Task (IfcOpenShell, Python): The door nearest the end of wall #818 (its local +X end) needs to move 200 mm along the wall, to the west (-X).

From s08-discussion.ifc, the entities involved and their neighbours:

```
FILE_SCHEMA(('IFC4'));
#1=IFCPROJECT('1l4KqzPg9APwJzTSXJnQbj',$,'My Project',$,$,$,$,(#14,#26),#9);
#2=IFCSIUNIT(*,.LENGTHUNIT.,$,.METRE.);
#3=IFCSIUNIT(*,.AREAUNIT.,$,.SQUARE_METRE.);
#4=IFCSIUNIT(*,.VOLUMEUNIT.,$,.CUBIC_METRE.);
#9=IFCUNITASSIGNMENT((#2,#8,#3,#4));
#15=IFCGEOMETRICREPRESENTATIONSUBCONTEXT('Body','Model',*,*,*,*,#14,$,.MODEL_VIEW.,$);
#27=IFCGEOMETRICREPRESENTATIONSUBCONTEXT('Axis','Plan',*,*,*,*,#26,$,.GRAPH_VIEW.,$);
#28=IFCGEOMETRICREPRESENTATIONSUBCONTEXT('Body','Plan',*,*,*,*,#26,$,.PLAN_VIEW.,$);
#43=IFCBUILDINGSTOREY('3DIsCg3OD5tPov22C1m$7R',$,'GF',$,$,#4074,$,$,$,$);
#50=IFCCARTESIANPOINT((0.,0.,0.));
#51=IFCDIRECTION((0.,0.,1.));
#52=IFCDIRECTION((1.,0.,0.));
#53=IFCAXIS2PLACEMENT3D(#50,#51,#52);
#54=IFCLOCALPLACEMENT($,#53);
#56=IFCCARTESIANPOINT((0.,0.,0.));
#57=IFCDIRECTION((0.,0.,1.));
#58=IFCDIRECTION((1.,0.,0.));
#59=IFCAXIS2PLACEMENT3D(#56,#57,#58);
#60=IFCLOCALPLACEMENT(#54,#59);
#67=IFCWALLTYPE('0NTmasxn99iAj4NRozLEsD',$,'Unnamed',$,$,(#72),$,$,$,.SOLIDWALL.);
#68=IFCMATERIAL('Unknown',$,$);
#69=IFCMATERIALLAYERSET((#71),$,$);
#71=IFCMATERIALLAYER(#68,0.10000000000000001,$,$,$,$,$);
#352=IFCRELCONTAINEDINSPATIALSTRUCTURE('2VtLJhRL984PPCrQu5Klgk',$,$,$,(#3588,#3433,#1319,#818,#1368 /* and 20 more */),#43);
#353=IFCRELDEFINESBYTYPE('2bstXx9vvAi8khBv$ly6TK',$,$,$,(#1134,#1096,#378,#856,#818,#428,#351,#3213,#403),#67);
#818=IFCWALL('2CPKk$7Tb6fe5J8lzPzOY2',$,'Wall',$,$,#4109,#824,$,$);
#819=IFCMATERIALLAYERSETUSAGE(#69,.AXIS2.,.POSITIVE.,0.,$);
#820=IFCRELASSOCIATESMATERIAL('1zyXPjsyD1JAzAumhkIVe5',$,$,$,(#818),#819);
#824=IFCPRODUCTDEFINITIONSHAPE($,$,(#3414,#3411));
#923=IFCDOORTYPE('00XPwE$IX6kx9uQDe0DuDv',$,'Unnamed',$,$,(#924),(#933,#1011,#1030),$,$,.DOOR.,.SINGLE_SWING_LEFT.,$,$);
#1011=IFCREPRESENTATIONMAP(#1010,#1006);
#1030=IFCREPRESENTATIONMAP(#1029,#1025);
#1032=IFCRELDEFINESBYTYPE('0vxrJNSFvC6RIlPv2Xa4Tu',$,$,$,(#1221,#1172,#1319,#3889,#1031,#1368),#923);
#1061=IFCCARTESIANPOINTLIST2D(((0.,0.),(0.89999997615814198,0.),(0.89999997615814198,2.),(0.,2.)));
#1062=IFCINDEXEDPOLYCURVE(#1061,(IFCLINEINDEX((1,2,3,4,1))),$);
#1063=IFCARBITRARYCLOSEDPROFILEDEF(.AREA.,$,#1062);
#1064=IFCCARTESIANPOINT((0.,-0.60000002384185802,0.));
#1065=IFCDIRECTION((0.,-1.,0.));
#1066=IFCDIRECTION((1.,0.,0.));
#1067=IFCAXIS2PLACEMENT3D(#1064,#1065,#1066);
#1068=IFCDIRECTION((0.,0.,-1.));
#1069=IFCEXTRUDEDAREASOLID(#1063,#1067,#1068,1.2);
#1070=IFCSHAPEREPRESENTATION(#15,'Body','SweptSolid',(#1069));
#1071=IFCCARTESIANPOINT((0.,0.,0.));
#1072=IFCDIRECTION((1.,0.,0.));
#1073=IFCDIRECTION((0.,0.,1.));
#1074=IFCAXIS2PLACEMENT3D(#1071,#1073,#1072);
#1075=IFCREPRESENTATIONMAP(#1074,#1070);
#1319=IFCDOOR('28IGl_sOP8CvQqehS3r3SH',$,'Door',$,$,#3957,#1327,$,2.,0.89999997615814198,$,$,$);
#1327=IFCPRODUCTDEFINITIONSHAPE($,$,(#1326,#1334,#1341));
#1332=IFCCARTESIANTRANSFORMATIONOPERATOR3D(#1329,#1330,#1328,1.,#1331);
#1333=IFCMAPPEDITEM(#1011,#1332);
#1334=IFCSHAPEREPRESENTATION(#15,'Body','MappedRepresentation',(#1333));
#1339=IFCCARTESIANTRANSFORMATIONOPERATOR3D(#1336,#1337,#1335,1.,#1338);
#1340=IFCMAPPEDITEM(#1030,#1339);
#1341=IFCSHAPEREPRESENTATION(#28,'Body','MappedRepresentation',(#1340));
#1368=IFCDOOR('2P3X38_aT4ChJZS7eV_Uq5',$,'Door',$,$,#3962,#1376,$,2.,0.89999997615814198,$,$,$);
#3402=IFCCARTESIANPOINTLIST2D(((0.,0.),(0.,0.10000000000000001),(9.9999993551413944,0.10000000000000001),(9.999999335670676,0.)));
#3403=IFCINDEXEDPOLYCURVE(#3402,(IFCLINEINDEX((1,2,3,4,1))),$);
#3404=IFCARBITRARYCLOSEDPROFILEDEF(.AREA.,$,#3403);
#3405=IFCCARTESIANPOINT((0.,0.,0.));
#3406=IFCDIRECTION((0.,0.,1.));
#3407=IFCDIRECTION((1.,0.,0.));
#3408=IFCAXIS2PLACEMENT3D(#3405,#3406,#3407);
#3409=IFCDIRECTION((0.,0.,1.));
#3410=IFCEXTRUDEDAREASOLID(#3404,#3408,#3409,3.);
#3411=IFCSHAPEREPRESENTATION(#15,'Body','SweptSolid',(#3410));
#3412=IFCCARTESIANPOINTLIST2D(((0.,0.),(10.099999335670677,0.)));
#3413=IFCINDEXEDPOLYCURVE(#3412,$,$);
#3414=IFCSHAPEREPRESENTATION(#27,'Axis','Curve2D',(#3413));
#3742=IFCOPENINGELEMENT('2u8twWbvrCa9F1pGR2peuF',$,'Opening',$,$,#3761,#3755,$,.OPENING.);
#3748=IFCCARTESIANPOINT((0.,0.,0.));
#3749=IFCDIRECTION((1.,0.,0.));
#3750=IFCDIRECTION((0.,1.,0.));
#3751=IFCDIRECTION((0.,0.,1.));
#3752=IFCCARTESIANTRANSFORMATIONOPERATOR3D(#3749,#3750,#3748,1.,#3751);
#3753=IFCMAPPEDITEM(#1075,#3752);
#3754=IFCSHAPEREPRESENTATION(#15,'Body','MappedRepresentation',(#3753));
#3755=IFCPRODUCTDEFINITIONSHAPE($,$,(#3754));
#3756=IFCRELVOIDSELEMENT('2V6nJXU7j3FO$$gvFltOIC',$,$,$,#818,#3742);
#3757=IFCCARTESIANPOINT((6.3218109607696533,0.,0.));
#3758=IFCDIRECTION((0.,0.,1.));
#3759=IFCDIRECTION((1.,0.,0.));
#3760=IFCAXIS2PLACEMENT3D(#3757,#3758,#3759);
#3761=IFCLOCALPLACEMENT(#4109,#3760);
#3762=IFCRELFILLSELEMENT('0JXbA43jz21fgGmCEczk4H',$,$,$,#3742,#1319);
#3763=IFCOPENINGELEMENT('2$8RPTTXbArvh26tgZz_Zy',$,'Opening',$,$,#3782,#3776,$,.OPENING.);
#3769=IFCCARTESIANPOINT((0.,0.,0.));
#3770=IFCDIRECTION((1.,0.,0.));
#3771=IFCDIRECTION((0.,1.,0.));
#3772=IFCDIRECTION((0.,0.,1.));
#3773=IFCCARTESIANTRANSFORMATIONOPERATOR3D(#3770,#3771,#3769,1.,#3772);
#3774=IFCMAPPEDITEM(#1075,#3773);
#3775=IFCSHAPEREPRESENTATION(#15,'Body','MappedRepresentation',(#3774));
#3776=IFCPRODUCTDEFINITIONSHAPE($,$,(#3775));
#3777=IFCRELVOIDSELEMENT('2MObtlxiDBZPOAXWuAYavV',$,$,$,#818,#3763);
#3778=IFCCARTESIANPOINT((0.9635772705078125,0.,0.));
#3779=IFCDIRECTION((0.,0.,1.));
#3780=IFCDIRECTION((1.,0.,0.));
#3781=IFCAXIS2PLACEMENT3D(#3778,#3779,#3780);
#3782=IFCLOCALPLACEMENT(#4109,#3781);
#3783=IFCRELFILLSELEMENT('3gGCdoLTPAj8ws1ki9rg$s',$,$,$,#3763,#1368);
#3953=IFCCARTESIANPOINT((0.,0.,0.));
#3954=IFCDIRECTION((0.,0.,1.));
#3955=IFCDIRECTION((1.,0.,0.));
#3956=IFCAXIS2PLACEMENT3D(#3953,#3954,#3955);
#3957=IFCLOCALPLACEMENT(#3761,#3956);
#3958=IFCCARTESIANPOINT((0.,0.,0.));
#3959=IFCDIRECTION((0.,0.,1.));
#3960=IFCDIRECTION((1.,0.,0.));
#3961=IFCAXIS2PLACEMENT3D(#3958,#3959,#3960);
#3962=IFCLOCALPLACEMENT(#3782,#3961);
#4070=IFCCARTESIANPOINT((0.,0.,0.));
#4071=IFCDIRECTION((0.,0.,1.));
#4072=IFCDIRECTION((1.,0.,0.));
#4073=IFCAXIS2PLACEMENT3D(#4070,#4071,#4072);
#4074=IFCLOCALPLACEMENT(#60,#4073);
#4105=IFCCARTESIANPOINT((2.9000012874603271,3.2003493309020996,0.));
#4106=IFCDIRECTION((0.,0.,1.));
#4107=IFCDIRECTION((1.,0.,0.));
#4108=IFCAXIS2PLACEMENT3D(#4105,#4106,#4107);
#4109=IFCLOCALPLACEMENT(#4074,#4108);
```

```python
import ifcopenshell
import ifcopenshell.api.geometry
import ifcopenshell.util.placement
import ifcopenshell.util.unit

model = ifcopenshell.open("s08-discussion.ifc")
unit_scale = ifcopenshell.util.unit.calculate_unit_scale(model)

door = model.by_guid("28IGl_sOP8CvQqehS3r3SH")
opening = door.FillsVoids[0].RelatingOpeningElement
wall = opening.VoidsElements[0].RelatingBuildingElement

wall_matrix = ifcopenshell.util.placement.get_local_placement(wall.ObjectPlacement)
shift = wall_matrix[:3, 0] * -0.2 / unit_scale
before = ifcopenshell.util.placement.get_local_placement(door.ObjectPlacement)[:3, 3].copy()

# The door is placed relative to its opening, so it follows when the opening moves.
matrix = ifcopenshell.util.placement.get_local_placement(opening.ObjectPlacement)
matrix[:3, 3] += shift
ifcopenshell.api.geometry.edit_object_placement(
    model, product=opening, matrix=matrix, is_si=False, should_transform_children=True
)

after = ifcopenshell.util.placement.get_local_placement(door.ObjectPlacement)[:3, 3]
print("door moved by", (after - before).round(3) + 0.0)

model.write("s08-discussion_rev.ifc")
```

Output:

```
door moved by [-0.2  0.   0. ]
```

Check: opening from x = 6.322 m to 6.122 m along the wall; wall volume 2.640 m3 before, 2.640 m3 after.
